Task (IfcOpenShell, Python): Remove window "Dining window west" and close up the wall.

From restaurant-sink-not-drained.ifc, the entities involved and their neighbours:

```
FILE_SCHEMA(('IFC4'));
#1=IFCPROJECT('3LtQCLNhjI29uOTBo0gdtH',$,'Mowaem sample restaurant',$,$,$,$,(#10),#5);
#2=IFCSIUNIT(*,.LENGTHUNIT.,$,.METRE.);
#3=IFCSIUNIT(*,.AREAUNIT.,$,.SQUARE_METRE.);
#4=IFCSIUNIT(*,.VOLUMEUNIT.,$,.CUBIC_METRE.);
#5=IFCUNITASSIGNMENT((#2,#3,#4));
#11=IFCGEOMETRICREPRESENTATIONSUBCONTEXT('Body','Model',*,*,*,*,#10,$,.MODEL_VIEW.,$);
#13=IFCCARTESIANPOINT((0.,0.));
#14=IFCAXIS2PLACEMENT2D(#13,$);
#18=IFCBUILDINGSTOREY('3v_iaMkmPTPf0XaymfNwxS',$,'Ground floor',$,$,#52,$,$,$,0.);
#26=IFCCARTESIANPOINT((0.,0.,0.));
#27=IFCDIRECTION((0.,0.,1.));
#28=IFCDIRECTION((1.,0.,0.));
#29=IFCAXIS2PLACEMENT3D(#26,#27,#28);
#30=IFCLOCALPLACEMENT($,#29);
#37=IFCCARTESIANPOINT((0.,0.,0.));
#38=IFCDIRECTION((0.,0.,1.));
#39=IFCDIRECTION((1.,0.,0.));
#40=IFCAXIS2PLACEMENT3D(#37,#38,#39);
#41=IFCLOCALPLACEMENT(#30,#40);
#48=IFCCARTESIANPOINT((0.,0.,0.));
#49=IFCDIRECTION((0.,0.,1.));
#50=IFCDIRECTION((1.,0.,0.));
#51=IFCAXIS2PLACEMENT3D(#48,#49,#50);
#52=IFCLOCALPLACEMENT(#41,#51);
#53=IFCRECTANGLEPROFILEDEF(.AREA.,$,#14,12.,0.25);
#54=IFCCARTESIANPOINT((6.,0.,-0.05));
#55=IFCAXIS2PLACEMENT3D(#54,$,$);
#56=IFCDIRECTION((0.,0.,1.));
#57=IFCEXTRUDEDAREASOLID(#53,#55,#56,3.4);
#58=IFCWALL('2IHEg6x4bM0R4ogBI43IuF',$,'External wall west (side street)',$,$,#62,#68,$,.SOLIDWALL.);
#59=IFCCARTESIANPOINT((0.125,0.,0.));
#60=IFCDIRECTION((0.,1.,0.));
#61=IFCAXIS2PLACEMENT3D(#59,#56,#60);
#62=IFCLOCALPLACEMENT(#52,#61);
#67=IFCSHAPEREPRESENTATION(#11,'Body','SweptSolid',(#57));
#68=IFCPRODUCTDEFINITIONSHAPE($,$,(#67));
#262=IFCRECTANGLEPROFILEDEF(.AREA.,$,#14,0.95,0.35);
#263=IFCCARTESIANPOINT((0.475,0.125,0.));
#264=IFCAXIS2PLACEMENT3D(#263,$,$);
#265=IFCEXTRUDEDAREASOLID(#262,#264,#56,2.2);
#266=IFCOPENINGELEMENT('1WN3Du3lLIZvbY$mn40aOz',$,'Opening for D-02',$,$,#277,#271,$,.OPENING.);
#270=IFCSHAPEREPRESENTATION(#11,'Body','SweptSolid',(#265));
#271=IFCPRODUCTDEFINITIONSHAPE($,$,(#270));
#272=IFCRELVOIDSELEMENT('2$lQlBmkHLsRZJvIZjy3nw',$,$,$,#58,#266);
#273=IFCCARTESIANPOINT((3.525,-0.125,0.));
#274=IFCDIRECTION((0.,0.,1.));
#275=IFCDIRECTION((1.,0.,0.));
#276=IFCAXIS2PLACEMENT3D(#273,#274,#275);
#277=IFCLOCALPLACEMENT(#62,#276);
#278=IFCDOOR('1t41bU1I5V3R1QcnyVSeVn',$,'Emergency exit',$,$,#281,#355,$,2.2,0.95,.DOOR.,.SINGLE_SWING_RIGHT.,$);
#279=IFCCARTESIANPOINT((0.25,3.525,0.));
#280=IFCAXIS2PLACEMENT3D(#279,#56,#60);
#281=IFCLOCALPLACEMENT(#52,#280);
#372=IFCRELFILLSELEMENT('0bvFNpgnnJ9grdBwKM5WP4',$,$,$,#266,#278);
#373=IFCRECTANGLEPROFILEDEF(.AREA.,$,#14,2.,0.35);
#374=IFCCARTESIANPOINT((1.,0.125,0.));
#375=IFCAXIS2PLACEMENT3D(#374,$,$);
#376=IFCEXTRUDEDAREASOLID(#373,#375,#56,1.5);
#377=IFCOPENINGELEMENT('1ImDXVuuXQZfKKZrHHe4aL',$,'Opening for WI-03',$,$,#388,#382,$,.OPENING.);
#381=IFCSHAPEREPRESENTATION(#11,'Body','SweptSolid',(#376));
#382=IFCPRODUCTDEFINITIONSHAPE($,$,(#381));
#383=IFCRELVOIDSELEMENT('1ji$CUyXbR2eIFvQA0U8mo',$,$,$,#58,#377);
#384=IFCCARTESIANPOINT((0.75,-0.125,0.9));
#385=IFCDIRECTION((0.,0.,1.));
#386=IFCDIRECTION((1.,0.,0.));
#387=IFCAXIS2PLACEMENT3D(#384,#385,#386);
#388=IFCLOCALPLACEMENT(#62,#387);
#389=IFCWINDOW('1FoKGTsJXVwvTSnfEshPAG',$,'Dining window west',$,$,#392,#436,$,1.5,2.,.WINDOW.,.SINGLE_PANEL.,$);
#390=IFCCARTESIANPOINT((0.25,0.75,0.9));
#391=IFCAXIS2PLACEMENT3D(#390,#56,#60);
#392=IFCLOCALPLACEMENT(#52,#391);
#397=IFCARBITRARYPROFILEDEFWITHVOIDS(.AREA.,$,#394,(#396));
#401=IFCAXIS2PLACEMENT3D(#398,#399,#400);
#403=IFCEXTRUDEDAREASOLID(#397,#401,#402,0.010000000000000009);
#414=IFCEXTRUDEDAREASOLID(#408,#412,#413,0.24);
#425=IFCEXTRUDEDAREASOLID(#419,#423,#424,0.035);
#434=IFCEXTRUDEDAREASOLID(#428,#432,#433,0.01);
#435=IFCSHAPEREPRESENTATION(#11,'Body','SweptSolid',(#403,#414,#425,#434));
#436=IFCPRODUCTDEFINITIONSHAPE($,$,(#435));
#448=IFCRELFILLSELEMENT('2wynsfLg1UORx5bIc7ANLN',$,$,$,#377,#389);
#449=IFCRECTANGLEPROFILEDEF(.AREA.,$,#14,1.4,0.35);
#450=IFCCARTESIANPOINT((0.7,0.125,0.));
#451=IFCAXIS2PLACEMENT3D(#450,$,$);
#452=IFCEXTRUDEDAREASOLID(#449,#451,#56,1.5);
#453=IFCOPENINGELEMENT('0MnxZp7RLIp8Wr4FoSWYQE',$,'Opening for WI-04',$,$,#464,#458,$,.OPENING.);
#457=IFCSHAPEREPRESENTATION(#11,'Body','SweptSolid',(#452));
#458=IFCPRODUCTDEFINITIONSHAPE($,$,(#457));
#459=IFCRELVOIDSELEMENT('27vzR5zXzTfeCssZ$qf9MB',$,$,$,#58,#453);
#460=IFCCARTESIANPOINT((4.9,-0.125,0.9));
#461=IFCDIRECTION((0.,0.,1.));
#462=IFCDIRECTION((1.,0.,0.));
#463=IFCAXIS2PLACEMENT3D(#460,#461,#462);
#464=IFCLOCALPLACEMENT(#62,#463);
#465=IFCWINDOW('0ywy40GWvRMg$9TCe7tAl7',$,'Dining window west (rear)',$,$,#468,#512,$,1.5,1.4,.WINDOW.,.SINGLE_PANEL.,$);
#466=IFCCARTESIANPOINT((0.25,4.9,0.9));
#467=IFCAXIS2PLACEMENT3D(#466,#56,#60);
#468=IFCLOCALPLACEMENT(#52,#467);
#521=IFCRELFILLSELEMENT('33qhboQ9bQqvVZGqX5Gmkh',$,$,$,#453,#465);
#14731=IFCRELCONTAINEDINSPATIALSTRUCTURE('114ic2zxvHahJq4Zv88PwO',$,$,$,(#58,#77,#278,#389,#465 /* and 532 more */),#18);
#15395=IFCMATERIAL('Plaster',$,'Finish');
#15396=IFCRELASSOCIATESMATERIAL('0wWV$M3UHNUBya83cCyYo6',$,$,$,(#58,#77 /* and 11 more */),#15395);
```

```python
import ifcopenshell
import ifcopenshell.api.feature
import ifcopenshell.api.root
import ifcopenshell.geom
import ifcopenshell.util.shape

model = ifcopenshell.open("restaurant-sink-not-drained.ifc")
settings = ifcopenshell.geom.settings()


def volume(element):
    """Net volume in cubic metres, openings subtracted."""
    shape = ifcopenshell.geom.create_shape(settings, element)
    return ifcopenshell.util.shape.get_volume(shape.geometry)


window = model.by_guid("1FoKGTsJXVwvTSnfEshPAG")
opening = window.FillsVoids[0].RelatingOpeningElement
wall = opening.VoidsElements[0].RelatingBuildingElement
before = volume(wall)

ifcopenshell.api.root.remove_product(model, product=window)
ifcopenshell.api.feature.remove_feature(model, feature=opening)

after = volume(wall)

print(f"wall volume {before:.3f} -> {after:.3f} m3")

model.write("restaurant-sink-not-drained_rev.ifc")
```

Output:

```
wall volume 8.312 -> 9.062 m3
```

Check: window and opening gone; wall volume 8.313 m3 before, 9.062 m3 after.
